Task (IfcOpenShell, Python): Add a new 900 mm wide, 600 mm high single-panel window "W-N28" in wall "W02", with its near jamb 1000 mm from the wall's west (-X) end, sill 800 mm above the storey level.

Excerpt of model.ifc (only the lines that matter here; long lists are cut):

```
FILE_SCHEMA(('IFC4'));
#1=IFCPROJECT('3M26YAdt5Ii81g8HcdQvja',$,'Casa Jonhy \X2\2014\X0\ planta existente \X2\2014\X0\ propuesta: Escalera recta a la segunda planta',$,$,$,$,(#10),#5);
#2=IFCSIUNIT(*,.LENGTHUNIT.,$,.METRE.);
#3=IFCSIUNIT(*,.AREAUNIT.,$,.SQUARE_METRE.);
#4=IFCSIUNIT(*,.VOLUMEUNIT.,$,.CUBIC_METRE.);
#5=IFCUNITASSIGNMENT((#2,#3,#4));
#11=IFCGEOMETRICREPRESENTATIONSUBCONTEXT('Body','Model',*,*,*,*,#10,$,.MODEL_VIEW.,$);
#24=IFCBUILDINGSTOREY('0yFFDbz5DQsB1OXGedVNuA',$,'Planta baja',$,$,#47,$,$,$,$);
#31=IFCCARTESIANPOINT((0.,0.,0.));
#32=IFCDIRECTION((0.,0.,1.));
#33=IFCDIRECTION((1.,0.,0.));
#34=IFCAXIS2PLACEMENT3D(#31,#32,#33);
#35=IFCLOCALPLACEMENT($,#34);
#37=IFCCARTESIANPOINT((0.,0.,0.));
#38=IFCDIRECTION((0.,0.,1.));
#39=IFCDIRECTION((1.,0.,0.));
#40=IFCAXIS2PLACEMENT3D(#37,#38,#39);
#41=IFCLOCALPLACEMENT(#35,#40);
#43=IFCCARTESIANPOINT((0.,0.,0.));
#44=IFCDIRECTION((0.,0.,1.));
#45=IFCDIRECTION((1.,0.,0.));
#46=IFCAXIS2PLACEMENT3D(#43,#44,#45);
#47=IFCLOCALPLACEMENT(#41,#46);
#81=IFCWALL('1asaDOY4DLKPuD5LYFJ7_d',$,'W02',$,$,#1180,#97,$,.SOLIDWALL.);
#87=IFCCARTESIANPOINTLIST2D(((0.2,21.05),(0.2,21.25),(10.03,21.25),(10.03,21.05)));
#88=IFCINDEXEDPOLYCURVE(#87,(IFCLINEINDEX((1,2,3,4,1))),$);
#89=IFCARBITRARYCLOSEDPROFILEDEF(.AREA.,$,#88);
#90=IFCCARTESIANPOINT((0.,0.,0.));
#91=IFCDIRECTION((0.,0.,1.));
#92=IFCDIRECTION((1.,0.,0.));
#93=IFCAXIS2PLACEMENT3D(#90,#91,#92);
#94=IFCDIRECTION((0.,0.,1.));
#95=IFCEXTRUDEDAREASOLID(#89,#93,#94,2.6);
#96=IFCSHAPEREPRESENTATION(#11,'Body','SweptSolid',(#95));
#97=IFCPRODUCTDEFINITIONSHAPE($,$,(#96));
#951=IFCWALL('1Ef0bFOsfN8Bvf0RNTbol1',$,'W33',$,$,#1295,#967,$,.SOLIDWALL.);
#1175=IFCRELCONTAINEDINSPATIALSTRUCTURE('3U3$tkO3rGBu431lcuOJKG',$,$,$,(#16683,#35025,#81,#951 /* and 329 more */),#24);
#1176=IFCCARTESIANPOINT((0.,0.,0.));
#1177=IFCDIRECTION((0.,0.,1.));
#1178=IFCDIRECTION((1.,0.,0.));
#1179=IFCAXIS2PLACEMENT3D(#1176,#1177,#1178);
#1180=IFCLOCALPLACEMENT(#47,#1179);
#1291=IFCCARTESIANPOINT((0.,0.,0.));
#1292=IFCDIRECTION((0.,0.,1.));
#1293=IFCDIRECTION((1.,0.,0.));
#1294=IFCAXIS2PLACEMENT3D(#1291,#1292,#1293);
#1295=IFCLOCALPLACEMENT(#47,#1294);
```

```python
import numpy as np
import ifcopenshell
import ifcopenshell.api.feature
import ifcopenshell.api.geometry
import ifcopenshell.api.root
import ifcopenshell.api.spatial
import ifcopenshell.geom
import ifcopenshell.util.element
import ifcopenshell.util.placement
import ifcopenshell.util.representation
import ifcopenshell.util.shape
import ifcopenshell.util.unit

model = ifcopenshell.open("model.ifc")
unit_scale = ifcopenshell.util.unit.calculate_unit_scale(model)
settings = ifcopenshell.geom.settings()


def volume(element):
    """Net volume in cubic metres, openings subtracted."""
    shape = ifcopenshell.geom.create_shape(settings, element)
    return ifcopenshell.util.shape.get_volume(shape.geometry)


wall = model.by_id(81)
storey = ifcopenshell.util.element.get_container(wall, ifc_class="IfcBuildingStorey")
context = ifcopenshell.util.representation.get_context(model, "Model", "Body", "MODEL_VIEW")
before = volume(wall)

width, height, from_end, sill = 0.9, 0.6, 1, 0.8  # metres

# The wall runs along its own X axis, and the end named is its -X end.
wall_shape = ifcopenshell.geom.create_shape(settings, wall)
x, y, z = ifcopenshell.util.shape.get_vertices(wall_shape.geometry).T
start = x.min() + from_end
face, thickness = float(y.min()), float(y.max() - y.min())
wall_matrix = ifcopenshell.util.placement.get_local_placement(wall.ObjectPlacement)
level = ifcopenshell.util.placement.get_local_placement(storey.ObjectPlacement)[2, 3]


def in_wall(x, y):
    """Placement at x, y metres in the wall's axes, at sill height."""
    matrix = wall_matrix.copy()
    matrix[:, 3] = wall_matrix @ np.array([x / unit_scale, y / unit_scale, 0.0, 1.0])
    matrix[2, 3] = level + sill / unit_scale
    return matrix


# Opening: a box that overshoots both wall faces by 50 mm.
opening = ifcopenshell.api.root.create_entity(model, ifc_class="IfcOpeningElement", predefined_type="OPENING")
box = ifcopenshell.api.geometry.add_wall_representation(
    model, context=context, length=width, height=height, thickness=thickness + 0.1
)
ifcopenshell.api.geometry.assign_representation(model, product=opening, representation=box)
ifcopenshell.api.geometry.edit_object_placement(model, product=opening, matrix=in_wall(start, face - 0.05), is_si=False)
ifcopenshell.api.feature.add_feature(model, feature=opening, element=wall)

window = ifcopenshell.api.root.create_entity(model, ifc_class="IfcWindow", name="W-N28", predefined_type="WINDOW")
window.OverallWidth, window.OverallHeight = width / unit_scale, height / unit_scale
window.PartitioningType = "SINGLE_PANEL"
body = ifcopenshell.api.geometry.add_window_representation(
    model,
    context=context,
    overall_width=window.OverallWidth,
    overall_height=window.OverallHeight,
    partition_type="SINGLE_PANEL",
)
ifcopenshell.api.geometry.assign_representation(model, product=window, representation=body)
ifcopenshell.api.spatial.assign_container(model, products=[window], relating_structure=storey)
ifcopenshell.api.feature.add_filling(model, opening=opening, element=window)

# Centre the window in the wall's thickness.
ifcopenshell.api.geometry.edit_object_placement(model, product=window, matrix=in_wall(start, face), is_si=False)
window_shape = ifcopenshell.geom.create_shape(settings, window)
depth = ifcopenshell.util.shape.get_vertices(window_shape.geometry)[:, 1]
offset = face + thickness / 2 - (depth.min() + depth.max()) / 2
ifcopenshell.api.geometry.edit_object_placement(model, product=window, matrix=in_wall(start, offset), is_si=False)

after = volume(wall)

print(f"wall volume {before:.3f} -> {after:.3f} m3")

model.write("model_v2.ifc")
```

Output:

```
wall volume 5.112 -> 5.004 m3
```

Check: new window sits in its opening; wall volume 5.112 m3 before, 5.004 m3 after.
